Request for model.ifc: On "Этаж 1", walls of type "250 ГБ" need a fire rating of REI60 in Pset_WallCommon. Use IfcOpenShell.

First a look at what the model holds.

```python
import ifcopenshell
import ifcopenshell.util.element

model = ifcopenshell.open("model.ifc")
print(model.schema)
storey = next(s for s in model.by_type("IfcBuildingStorey") if s.Name == "Этаж 1")
walls = [e for e in ifcopenshell.util.element.get_decomposition(storey) if e.is_a("IfcWall")]
seen = {}
for e in walls:
    element_type = ifcopenshell.util.element.get_type(e)
    key = (element_type.Name if element_type != e and element_type else None, ifcopenshell.util.element.get_pset(e, "Pset_WallCommon", "FireRating"))
    seen[key] = seen.get(key, 0) + 1
for (name, value), count in sorted(seen.items(), key=str):
    print(count, "x", name, "|", value)
```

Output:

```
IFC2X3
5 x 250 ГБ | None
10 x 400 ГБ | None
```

```python
import ifcopenshell
import ifcopenshell.api.pset
import ifcopenshell.util.element

model = ifcopenshell.open("model.ifc")

storey = next(s for s in model.by_type("IfcBuildingStorey") if s.Name == "Этаж 1")
walls = [e for e in ifcopenshell.util.element.get_decomposition(storey) if e.is_a("IfcWall")]

count = 0
for e in walls:
    element_type = ifcopenshell.util.element.get_type(e)
    if element_type in (None, e) or element_type.Name != "250 ГБ":
        continue
    # add_pset returns the element's existing set when there is one.
    pset = ifcopenshell.api.pset.add_pset(model, product=e, name="Pset_WallCommon")
    ifcopenshell.api.pset.edit_pset(model, pset=pset, properties={"FireRating": "REI60"})
    count += 1

print(count, "walls updated")

model.write("model-out.ifc")
```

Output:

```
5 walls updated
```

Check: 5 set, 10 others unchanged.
